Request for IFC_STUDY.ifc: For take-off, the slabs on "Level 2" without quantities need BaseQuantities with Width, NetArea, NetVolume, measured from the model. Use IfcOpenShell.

First a look at what the model holds.

```python
import ifcopenshell
import ifcopenshell.util.element
import ifcopenshell.util.unit

model = ifcopenshell.open("IFC_STUDY.ifc")
print(model.schema)
for unit_type in ("LENGTHUNIT", "AREAUNIT", "VOLUMEUNIT"):
    print(unit_type, ifcopenshell.util.unit.calculate_unit_scale(model, unit_type))
storey = next(s for s in model.by_type("IfcBuildingStorey") if s.Name == "Level 2")
slabs = [e for e in ifcopenshell.util.element.get_decomposition(storey) if e.is_a("IfcSlab")]
for e in sorted(slabs, key=lambda e: e.id()):
    print(e.id(), e.is_a(), e.Name, list(ifcopenshell.util.element.get_psets(e, qtos_only=True)), sep=" | ")
```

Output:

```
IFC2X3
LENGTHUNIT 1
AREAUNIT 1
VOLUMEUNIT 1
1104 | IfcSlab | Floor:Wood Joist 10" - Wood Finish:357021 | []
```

```python
import ifcopenshell
import ifcopenshell.api.pset
import ifcopenshell.geom
import ifcopenshell.util.element
import ifcopenshell.util.shape
import ifcopenshell.util.unit

model = ifcopenshell.open("IFC_STUDY.ifc")
unit_scale = ifcopenshell.util.unit.calculate_unit_scale(model)
area_scale = ifcopenshell.util.unit.calculate_unit_scale(model, "AREAUNIT")
volume_scale = ifcopenshell.util.unit.calculate_unit_scale(model, "VOLUMEUNIT")
settings = ifcopenshell.geom.settings()

storey = next(s for s in model.by_type("IfcBuildingStorey") if s.Name == "Level 2")
slabs = [e for e in ifcopenshell.util.element.get_decomposition(storey) if e.is_a("IfcSlab")]

for e in sorted(slabs, key=lambda e: e.id()):
    if ifcopenshell.util.element.get_psets(e, qtos_only=True, should_inherit=False):
        continue
    # Geometry comes back in metres, in the element's own axes.
    shape = ifcopenshell.geom.create_shape(settings, e)
    values = {
        "Width": ifcopenshell.util.shape.get_z(shape.geometry) / unit_scale,
        "NetArea": ifcopenshell.util.shape.get_footprint_area(shape.geometry) / area_scale,
        "NetVolume": ifcopenshell.util.shape.get_volume(shape.geometry) / volume_scale,
    }
    qto = ifcopenshell.api.pset.add_qto(model, product=e, name="BaseQuantities")
    ifcopenshell.api.pset.edit_qto(model, qto=qto, properties=values)
    print(e.id(), {k: round(v, 3) for k, v in values.items()})

model.write("IFC_STUDY-out.ifc")
```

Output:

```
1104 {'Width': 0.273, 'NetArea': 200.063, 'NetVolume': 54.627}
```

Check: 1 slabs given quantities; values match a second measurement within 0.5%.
